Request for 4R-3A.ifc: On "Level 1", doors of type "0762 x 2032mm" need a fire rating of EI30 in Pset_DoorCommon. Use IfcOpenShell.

First a look at what the model holds.

```python
import ifcopenshell
import ifcopenshell.util.element

model = ifcopenshell.open("4R-3A.ifc")
print(model.schema)
storey = next(s for s in model.by_type("IfcBuildingStorey") if s.Name == "Level 1")
doors = [e for e in ifcopenshell.util.element.get_decomposition(storey) if e.is_a("IfcDoor")]
seen = {}
for e in doors:
    element_type = ifcopenshell.util.element.get_type(e)
    key = (element_type.Name if element_type != e and element_type else None, ifcopenshell.util.element.get_pset(e, "Pset_DoorCommon", "FireRating"))
    seen[key] = seen.get(key, 0) + 1
for (name, value), count in sorted(seen.items(), key=str):
    print(count, "x", name, "|", value)
```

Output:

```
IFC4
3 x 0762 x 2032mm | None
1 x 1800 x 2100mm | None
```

```python
import ifcopenshell
import ifcopenshell.api.pset
import ifcopenshell.util.element

model = ifcopenshell.open("4R-3A.ifc")

storey = next(s for s in model.by_type("IfcBuildingStorey") if s.Name == "Level 1")
doors = [e for e in ifcopenshell.util.element.get_decomposition(storey) if e.is_a("IfcDoor")]

count = 0
for e in doors:
    element_type = ifcopenshell.util.element.get_type(e)
    if element_type in (None, e) or element_type.Name != "0762 x 2032mm":
        continue
    # add_pset returns the element's existing set when there is one.
    pset = ifcopenshell.api.pset.add_pset(model, product=e, name="Pset_DoorCommon")
    ifcopenshell.api.pset.edit_pset(model, pset=pset, properties={"FireRating": "EI30"})
    count += 1

print(count, "doors updated")

model.write("4R-3A_v2.ifc")
```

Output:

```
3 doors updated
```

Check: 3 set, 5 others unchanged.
